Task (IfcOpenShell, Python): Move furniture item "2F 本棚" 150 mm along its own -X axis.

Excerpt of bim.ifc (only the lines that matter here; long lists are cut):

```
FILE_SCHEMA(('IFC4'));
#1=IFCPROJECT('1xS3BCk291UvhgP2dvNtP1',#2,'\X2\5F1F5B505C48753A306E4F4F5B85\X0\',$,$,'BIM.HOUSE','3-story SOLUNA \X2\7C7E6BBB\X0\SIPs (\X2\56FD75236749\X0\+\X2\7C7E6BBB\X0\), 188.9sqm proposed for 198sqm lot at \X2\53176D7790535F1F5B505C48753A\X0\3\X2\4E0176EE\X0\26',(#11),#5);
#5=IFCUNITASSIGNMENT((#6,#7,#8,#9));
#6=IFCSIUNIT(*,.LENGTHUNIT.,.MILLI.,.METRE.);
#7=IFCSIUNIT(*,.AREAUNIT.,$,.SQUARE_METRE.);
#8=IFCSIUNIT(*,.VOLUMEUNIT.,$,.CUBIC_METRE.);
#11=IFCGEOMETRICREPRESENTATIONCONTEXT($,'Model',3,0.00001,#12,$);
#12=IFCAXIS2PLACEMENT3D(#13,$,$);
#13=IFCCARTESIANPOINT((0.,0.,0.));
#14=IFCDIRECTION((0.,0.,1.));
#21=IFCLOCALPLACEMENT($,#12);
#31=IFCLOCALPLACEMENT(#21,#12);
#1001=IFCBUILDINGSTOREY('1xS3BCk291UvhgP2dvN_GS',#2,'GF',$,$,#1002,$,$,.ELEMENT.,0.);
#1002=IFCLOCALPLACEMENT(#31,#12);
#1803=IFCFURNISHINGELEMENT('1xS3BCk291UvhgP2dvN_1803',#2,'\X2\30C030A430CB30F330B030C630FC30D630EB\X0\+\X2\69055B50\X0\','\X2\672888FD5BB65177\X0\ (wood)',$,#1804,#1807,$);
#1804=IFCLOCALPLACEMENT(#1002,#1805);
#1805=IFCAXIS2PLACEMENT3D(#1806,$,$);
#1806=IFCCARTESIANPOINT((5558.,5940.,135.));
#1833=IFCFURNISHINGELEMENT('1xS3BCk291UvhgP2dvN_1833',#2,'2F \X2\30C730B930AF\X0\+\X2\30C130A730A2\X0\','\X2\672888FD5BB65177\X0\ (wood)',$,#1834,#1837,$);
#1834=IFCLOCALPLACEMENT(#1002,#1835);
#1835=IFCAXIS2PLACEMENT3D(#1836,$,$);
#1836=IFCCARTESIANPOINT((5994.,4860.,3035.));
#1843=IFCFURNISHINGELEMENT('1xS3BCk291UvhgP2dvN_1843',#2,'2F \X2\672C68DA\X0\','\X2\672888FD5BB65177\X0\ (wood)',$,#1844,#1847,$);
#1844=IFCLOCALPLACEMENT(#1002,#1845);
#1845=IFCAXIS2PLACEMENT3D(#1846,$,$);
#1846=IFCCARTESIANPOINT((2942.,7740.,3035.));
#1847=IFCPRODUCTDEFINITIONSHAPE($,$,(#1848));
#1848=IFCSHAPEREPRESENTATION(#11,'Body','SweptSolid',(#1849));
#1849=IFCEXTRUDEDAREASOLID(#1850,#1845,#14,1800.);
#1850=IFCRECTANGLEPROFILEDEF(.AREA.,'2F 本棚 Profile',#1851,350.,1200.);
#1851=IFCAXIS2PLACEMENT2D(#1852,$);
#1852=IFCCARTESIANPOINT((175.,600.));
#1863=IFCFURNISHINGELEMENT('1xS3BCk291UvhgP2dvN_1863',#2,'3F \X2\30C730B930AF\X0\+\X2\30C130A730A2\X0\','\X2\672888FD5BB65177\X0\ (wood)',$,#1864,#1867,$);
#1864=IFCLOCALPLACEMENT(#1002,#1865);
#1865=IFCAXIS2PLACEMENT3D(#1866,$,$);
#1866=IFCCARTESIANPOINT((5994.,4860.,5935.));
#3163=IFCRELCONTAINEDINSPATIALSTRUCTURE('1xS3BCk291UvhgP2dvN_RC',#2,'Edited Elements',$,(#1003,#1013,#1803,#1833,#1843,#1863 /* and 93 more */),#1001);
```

```python
import ifcopenshell
import ifcopenshell.api.geometry
import ifcopenshell.util.placement

model = ifcopenshell.open("bim.ifc")

item = model.by_id(1843)
matrix = ifcopenshell.util.placement.get_local_placement(item.ObjectPlacement)
matrix[:3, 3] -= matrix[:3, 0] * 150.0
ifcopenshell.api.geometry.edit_object_placement(model, product=item, matrix=matrix, is_si=False)

print(ifcopenshell.util.placement.get_local_placement(item.ObjectPlacement).round(3) + 0.0)

model.write("bim-out.ifc")
```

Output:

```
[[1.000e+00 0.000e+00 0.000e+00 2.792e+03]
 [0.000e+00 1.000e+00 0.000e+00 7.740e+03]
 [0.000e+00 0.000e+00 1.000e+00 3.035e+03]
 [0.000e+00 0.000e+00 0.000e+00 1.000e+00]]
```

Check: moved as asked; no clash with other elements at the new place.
